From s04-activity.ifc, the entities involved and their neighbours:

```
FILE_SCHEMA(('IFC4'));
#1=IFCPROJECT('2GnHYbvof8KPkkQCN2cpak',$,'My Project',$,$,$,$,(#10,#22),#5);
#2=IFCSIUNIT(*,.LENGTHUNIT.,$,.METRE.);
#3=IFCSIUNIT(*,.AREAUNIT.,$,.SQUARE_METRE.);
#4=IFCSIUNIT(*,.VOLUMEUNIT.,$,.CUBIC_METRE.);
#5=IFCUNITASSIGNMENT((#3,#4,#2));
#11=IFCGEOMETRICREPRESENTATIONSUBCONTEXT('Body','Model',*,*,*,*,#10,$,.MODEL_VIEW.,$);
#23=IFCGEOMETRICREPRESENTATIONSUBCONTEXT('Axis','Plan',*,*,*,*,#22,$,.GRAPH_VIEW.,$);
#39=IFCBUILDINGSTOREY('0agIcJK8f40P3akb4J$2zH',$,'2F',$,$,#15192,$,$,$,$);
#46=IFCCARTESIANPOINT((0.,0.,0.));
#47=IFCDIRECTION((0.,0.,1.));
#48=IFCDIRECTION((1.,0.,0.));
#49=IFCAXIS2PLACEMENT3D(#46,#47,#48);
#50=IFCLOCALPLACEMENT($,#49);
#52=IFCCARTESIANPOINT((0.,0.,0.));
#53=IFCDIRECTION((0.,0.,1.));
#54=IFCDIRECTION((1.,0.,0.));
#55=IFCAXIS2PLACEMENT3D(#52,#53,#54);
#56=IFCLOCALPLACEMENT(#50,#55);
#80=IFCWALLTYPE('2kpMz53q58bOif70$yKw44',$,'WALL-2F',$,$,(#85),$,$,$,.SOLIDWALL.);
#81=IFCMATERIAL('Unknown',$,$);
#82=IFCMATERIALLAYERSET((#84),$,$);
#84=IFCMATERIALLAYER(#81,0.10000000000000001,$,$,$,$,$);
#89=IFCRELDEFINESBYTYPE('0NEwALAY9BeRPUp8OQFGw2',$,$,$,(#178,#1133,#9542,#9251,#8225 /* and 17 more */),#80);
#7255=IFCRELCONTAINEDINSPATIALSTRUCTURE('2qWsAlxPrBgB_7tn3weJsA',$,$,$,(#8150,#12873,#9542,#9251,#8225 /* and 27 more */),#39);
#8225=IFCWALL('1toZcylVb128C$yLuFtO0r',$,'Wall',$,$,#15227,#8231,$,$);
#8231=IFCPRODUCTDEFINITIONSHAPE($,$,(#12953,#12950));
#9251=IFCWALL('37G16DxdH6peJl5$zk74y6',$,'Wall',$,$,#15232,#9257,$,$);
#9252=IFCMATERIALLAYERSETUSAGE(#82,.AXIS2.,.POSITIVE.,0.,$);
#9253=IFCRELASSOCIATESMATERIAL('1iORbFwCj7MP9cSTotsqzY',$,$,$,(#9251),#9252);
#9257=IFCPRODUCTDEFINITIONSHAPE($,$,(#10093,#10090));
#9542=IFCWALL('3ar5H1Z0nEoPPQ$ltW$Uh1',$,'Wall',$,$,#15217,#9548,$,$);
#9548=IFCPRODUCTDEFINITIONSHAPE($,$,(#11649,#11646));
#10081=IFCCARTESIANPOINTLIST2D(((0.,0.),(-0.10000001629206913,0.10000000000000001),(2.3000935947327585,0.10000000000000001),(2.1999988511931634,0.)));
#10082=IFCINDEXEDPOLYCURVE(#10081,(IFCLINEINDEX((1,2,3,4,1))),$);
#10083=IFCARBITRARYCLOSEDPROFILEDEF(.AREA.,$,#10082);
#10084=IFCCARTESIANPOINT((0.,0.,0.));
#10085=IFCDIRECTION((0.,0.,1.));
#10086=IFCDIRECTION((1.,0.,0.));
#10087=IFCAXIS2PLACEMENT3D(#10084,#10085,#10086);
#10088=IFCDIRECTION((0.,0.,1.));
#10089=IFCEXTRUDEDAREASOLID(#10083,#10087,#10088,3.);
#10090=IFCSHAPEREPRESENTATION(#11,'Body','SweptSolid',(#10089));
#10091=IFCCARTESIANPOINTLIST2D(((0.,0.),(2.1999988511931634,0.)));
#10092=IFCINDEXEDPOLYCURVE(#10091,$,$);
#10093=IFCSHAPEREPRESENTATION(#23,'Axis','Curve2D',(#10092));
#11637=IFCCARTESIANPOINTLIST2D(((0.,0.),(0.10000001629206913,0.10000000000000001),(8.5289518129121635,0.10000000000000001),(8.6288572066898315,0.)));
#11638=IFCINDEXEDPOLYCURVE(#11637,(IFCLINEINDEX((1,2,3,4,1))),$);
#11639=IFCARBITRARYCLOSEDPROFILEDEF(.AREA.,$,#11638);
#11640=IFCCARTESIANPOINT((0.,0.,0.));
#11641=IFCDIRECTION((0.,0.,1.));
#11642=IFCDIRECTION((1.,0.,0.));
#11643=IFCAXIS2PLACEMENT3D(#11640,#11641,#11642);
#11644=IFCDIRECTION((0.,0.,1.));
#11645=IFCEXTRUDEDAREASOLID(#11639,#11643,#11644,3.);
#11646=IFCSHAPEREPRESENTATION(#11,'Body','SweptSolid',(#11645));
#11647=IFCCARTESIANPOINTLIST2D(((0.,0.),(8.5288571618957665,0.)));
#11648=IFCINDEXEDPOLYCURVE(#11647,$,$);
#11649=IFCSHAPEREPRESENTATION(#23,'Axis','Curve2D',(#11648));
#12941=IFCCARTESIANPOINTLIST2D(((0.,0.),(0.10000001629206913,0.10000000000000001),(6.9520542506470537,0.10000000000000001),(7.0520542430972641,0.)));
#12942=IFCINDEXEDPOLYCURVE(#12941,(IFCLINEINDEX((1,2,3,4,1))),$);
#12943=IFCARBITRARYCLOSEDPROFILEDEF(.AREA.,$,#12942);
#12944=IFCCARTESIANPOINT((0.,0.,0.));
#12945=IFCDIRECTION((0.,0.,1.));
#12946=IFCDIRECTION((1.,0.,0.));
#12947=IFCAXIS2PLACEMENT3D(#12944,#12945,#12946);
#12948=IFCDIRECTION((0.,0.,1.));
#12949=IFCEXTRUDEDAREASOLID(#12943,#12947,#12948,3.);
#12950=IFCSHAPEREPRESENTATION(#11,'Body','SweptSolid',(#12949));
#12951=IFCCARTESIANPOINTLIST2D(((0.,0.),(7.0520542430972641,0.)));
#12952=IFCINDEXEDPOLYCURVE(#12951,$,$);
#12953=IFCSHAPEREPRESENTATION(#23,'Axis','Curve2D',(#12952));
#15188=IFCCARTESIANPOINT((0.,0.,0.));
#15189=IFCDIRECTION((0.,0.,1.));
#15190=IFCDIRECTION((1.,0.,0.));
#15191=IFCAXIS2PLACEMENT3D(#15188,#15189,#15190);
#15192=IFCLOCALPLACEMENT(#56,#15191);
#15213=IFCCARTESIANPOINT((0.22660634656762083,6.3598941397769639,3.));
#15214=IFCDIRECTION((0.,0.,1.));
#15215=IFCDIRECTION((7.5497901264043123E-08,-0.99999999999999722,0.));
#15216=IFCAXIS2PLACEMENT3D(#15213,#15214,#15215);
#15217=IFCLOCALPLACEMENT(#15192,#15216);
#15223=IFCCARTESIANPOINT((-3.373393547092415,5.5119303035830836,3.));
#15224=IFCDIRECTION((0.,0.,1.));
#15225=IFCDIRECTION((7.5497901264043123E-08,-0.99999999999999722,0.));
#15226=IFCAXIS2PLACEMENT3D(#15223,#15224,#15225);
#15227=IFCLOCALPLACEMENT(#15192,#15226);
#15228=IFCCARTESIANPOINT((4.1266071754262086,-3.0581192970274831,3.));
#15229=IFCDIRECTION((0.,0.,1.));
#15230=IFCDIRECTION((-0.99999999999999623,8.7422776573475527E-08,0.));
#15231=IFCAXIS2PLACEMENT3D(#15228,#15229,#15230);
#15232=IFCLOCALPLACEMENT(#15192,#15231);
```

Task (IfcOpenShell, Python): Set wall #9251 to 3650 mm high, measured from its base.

```python
import ifcopenshell
import ifcopenshell.geom
import ifcopenshell.util.representation
import ifcopenshell.util.shape
import ifcopenshell.util.unit

model = ifcopenshell.open("s04-activity.ifc")
unit_scale = ifcopenshell.util.unit.calculate_unit_scale(model)
settings = ifcopenshell.geom.settings()


def volume(element):
    """Net volume in cubic metres, openings subtracted."""
    shape = ifcopenshell.geom.create_shape(settings, element)
    return ifcopenshell.util.shape.get_volume(shape.geometry)


wall = model.by_guid("37G16DxdH6peJl5$zk74y6")
before = volume(wall)

body = ifcopenshell.util.representation.get_representation(wall, "Model", "Body")
solid = body.Items[0]
old_height = solid.Depth
solid.Depth = 3.65 / unit_scale
after = volume(wall)

print(f"height {old_height:g} -> {solid.Depth:g}, volume {before:.3f} -> {after:.3f} m3")

model.write("s04-activity_v2.ifc")
```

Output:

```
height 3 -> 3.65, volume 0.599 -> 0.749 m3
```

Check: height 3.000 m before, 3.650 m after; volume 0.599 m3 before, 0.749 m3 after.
